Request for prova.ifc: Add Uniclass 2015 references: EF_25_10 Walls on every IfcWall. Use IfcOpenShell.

First a look at what the model holds.

```python
import ifcopenshell

model = ifcopenshell.open("prova.ifc")
print(model.schema)
print("classifications:", [c.Name for c in model.by_type("IfcClassification")])
for ifc_class in ("IfcDoor", "IfcRoof", "IfcStair", "IfcWall", "IfcWindow"):
    print(ifc_class, len(model.by_type(ifc_class)))
```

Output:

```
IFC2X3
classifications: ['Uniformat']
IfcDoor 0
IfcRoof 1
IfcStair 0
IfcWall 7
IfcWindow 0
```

```python
import ifcopenshell
import ifcopenshell.api.classification

model = ifcopenshell.open("prova.ifc")

# IFC2X3 requires Source and Edition and has no link from the project to the system.
system = model.create_entity("IfcClassification", Source="NBS", Edition="2015", Name="Uniclass 2015")

codes = {
    "IfcWall": ("EF_25_10", "Walls"),
}
for ifc_class, (code, name) in codes.items():
    products = model.by_type(ifc_class)
    ifcopenshell.api.classification.add_reference(
        model, products=products, classification=system, identification=code, name=name
    )
    print(code, len(products))

model.write("prova-out.ifc")
```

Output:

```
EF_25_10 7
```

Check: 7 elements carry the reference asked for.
